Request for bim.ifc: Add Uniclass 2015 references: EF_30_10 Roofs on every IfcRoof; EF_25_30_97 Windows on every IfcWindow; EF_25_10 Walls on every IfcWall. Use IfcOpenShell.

First a look at what the model holds.

```python
import ifcopenshell

model = ifcopenshell.open("bim.ifc")
print(model.schema)
print("classifications:", [c.Name for c in model.by_type("IfcClassification")])
for ifc_class in ("IfcDoor", "IfcRoof", "IfcStair", "IfcWall", "IfcWindow"):
    print(ifc_class, len(model.by_type(ifc_class)))
```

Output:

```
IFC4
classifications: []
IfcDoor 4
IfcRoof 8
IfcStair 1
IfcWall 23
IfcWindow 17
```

```python
import ifcopenshell
import ifcopenshell.api.classification

model = ifcopenshell.open("bim.ifc")

system = ifcopenshell.api.classification.add_classification(model, classification="Uniclass 2015")

codes = {
    "IfcRoof": ("EF_30_10", "Roofs"),
    "IfcWindow": ("EF_25_30_97", "Windows"),
    "IfcWall": ("EF_25_10", "Walls"),
}
for ifc_class, (code, name) in codes.items():
    products = model.by_type(ifc_class)
    ifcopenshell.api.classification.add_reference(
        model, products=products, classification=system, identification=code, name=name
    )
    print(code, len(products))

model.write("bim_rev.ifc")
```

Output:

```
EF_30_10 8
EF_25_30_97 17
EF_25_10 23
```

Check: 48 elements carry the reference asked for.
